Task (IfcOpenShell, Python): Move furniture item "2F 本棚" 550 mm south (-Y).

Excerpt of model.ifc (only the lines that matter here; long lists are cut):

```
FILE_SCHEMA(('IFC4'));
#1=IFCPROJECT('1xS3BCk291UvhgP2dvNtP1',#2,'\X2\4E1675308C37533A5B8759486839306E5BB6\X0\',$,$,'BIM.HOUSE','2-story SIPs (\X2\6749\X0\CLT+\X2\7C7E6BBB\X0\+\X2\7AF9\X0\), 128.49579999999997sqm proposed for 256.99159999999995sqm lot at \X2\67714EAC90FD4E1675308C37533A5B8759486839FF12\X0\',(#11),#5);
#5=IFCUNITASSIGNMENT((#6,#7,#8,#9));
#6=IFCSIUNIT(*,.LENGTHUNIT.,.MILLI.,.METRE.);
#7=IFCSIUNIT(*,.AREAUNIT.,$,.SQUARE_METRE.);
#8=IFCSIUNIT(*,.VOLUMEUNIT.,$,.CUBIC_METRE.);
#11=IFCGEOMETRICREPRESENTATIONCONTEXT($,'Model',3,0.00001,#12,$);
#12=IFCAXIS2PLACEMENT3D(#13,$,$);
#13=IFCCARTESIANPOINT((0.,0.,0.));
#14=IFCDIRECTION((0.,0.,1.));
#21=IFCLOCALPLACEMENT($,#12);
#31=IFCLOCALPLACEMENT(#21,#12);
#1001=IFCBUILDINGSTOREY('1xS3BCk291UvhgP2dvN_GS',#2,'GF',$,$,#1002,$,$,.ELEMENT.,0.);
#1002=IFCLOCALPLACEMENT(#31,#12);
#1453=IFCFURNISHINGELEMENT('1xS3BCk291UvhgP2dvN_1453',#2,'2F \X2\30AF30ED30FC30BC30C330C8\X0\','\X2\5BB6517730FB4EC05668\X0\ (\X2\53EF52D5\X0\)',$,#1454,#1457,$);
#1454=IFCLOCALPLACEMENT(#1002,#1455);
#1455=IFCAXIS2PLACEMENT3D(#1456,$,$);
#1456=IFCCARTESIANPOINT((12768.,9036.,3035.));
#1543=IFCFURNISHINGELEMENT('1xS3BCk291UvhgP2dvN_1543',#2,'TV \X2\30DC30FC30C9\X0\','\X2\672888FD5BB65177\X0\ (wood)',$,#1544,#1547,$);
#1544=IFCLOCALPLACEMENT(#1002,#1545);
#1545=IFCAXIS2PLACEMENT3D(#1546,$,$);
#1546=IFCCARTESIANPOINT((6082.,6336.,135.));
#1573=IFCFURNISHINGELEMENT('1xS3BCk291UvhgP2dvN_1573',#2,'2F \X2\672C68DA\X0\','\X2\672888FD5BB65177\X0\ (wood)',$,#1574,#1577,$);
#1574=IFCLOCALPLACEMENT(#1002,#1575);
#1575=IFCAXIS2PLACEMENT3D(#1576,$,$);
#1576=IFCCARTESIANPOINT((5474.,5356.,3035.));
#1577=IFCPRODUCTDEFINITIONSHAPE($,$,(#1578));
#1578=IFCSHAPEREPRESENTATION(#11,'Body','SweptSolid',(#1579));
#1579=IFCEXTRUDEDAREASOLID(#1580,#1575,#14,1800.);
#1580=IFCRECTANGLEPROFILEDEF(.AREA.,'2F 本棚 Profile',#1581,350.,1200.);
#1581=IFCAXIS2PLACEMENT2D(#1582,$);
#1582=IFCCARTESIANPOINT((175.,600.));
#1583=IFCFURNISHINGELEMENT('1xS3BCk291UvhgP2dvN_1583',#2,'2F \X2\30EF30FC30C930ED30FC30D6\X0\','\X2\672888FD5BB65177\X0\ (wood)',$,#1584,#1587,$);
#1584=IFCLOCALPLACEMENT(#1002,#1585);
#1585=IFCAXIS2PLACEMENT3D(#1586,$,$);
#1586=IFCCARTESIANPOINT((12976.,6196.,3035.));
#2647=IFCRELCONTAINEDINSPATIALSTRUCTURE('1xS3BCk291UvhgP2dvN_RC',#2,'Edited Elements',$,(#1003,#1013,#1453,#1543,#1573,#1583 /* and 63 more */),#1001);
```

```python
import ifcopenshell
import ifcopenshell.api.geometry
import ifcopenshell.util.placement
import ifcopenshell.util.unit

model = ifcopenshell.open("model.ifc")
unit_scale = ifcopenshell.util.unit.calculate_unit_scale(model)

item = model.by_id(1573)
matrix = ifcopenshell.util.placement.get_local_placement(item.ObjectPlacement)
matrix[1, 3] -= 0.55 / unit_scale
ifcopenshell.api.geometry.edit_object_placement(model, product=item, matrix=matrix, is_si=False)

print(ifcopenshell.util.placement.get_local_placement(item.ObjectPlacement).round(3) + 0.0)

model.write("model-out.ifc")
```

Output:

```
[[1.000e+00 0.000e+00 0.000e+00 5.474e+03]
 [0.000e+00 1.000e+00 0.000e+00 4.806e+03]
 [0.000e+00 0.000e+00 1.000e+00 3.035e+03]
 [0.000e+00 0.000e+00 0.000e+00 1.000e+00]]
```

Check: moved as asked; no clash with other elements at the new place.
